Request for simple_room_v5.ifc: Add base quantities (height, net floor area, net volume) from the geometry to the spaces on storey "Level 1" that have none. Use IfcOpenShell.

First a look at what the model holds.

```python
import ifcopenshell
import ifcopenshell.util.element
import ifcopenshell.util.unit

model = ifcopenshell.open("simple_room_v5.ifc")
print(model.schema)
for unit_type in ("LENGTHUNIT", "AREAUNIT", "VOLUMEUNIT"):
    print(unit_type, ifcopenshell.util.unit.calculate_unit_scale(model, unit_type))
storey = next(s for s in model.by_type("IfcBuildingStorey") if s.Name == "Level 1")
spaces = [e for e in ifcopenshell.util.element.get_decomposition(storey) if e.is_a("IfcSpace")]
for e in sorted(spaces, key=lambda e: e.id()):
    print(e.id(), e.is_a(), e.Name, list(ifcopenshell.util.element.get_psets(e, qtos_only=True)), sep=" | ")
```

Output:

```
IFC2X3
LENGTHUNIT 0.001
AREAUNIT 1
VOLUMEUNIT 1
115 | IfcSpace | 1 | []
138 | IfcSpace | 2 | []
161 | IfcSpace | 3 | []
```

```python
import ifcopenshell
import ifcopenshell.api.pset
import ifcopenshell.geom
import ifcopenshell.util.element
import ifcopenshell.util.shape
import ifcopenshell.util.unit

model = ifcopenshell.open("simple_room_v5.ifc")
unit_scale = ifcopenshell.util.unit.calculate_unit_scale(model)
area_scale = ifcopenshell.util.unit.calculate_unit_scale(model, "AREAUNIT")
volume_scale = ifcopenshell.util.unit.calculate_unit_scale(model, "VOLUMEUNIT")
settings = ifcopenshell.geom.settings()

storey = next(s for s in model.by_type("IfcBuildingStorey") if s.Name == "Level 1")
spaces = [e for e in ifcopenshell.util.element.get_decomposition(storey) if e.is_a("IfcSpace")]

for e in sorted(spaces, key=lambda e: e.id()):
    if ifcopenshell.util.element.get_psets(e, qtos_only=True, should_inherit=False):
        continue
    # Geometry comes back in metres, in the element's own axes.
    shape = ifcopenshell.geom.create_shape(settings, e)
    values = {
        "Height": ifcopenshell.util.shape.get_z(shape.geometry) / unit_scale,
        "NetFloorArea": ifcopenshell.util.shape.get_footprint_area(shape.geometry) / area_scale,
        "NetVolume": ifcopenshell.util.shape.get_volume(shape.geometry) / volume_scale,
    }
    qto = ifcopenshell.api.pset.add_qto(model, product=e, name="BaseQuantities")
    ifcopenshell.api.pset.edit_qto(model, qto=qto, properties=values)
    print(e.id(), {k: round(v, 3) for k, v in values.items()})

model.write("simple_room_v5-out.ifc")
```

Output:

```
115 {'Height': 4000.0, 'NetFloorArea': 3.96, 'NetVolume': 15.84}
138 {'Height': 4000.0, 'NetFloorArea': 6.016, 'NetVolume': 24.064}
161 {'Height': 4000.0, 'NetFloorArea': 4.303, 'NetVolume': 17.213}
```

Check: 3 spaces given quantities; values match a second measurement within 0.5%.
